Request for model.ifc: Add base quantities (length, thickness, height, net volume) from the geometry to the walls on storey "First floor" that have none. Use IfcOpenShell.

First a look at what the model holds.

```python
import ifcopenshell
import ifcopenshell.util.element
import ifcopenshell.util.unit

model = ifcopenshell.open("model.ifc")
print(model.schema)
for unit_type in ("LENGTHUNIT", "AREAUNIT", "VOLUMEUNIT"):
    print(unit_type, ifcopenshell.util.unit.calculate_unit_scale(model, unit_type))
storey = next(s for s in model.by_type("IfcBuildingStorey") if s.Name == "First floor")
walls = [e for e in ifcopenshell.util.element.get_decomposition(storey) if e.is_a("IfcWall")]
for e in sorted(walls, key=lambda e: e.id()):
    print(e.id(), e.is_a(), e.Name, list(ifcopenshell.util.element.get_psets(e, qtos_only=True)), sep=" | ")
```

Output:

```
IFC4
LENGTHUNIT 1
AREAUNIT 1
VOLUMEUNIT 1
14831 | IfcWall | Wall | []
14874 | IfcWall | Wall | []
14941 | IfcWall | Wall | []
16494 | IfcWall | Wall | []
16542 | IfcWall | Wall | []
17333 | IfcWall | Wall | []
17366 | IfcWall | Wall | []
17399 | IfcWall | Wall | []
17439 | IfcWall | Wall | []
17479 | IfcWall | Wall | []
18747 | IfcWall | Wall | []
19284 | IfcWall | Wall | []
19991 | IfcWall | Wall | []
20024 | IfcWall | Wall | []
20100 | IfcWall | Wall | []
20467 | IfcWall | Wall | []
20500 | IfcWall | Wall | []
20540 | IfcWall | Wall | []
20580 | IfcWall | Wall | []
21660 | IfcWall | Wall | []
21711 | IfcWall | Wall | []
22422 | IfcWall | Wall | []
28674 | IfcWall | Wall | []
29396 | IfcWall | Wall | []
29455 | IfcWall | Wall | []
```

```python
import ifcopenshell
import ifcopenshell.api.pset
import ifcopenshell.geom
import ifcopenshell.util.element
import ifcopenshell.util.shape
import ifcopenshell.util.unit

model = ifcopenshell.open("model.ifc")
unit_scale = ifcopenshell.util.unit.calculate_unit_scale(model)
volume_scale = ifcopenshell.util.unit.calculate_unit_scale(model, "VOLUMEUNIT")
settings = ifcopenshell.geom.settings()

storey = next(s for s in model.by_type("IfcBuildingStorey") if s.Name == "First floor")
walls = [e for e in ifcopenshell.util.element.get_decomposition(storey) if e.is_a("IfcWall")]

for e in sorted(walls, key=lambda e: e.id()):
    if ifcopenshell.util.element.get_psets(e, qtos_only=True, should_inherit=False):
        continue
    # Geometry comes back in metres, in the element's own axes.
    shape = ifcopenshell.geom.create_shape(settings, e)
    values = {
        "Length": ifcopenshell.util.shape.get_x(shape.geometry) / unit_scale,
        "Width": ifcopenshell.util.shape.get_y(shape.geometry) / unit_scale,
        "Height": ifcopenshell.util.shape.get_z(shape.geometry) / unit_scale,
        "NetVolume": ifcopenshell.util.shape.get_volume(shape.geometry) / volume_scale,
    }
    qto = ifcopenshell.api.pset.add_qto(model, product=e, name="Qto_WallBaseQuantities")
    ifcopenshell.api.pset.edit_qto(model, qto=qto, properties=values)
    print(e.id(), {k: round(v, 3) for k, v in values.items()})

model.write("model_updated.ifc")
```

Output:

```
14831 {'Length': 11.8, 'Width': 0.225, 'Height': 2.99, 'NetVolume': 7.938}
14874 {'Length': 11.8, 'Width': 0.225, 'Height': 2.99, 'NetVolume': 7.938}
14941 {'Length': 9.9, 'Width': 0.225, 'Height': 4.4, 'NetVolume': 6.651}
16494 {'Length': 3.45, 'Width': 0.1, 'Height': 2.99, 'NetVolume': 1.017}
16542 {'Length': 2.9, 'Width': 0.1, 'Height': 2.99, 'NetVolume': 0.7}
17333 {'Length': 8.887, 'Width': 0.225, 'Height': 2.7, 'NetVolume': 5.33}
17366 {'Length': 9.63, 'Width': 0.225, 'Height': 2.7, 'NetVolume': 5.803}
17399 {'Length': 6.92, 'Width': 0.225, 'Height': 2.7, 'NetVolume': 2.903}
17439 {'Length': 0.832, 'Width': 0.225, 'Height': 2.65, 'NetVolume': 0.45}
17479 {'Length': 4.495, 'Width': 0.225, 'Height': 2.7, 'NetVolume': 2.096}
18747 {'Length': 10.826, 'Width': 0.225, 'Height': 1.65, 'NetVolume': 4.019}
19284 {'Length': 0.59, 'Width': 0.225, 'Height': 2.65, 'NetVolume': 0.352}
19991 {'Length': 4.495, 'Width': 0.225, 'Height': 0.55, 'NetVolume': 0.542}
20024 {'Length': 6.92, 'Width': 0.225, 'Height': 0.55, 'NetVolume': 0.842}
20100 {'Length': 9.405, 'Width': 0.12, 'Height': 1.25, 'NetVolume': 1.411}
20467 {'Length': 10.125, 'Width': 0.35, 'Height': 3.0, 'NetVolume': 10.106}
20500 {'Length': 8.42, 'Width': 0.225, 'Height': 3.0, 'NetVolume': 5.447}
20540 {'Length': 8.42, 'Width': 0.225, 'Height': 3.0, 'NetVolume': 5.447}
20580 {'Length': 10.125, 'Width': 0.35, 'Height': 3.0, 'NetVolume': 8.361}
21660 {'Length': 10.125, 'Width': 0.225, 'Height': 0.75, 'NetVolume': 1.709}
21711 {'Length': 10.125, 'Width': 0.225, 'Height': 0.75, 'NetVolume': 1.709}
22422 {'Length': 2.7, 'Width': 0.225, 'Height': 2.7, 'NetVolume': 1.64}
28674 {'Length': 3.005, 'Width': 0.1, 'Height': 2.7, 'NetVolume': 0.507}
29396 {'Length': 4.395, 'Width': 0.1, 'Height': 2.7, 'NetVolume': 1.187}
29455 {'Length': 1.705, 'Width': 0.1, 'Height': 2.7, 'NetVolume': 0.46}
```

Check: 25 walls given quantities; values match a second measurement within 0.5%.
